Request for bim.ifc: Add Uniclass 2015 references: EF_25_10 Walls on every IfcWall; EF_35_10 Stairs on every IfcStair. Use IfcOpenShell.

First a look at what the model holds.

```python
import ifcopenshell

model = ifcopenshell.open("bim.ifc")
print(model.schema)
print("classifications:", [c.Name for c in model.by_type("IfcClassification")])
for ifc_class in ("IfcDoor", "IfcRoof", "IfcStair", "IfcWall", "IfcWindow"):
    print(ifc_class, len(model.by_type(ifc_class)))
```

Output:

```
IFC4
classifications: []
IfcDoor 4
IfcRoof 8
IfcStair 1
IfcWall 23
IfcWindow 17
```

```python
import ifcopenshell
import ifcopenshell.api.classification

model = ifcopenshell.open("bim.ifc")

system = ifcopenshell.api.classification.add_classification(model, classification="Uniclass 2015")

codes = {
    "IfcWall": ("EF_25_10", "Walls"),
    "IfcStair": ("EF_35_10", "Stairs"),
}
for ifc_class, (code, name) in codes.items():
    products = model.by_type(ifc_class)
    ifcopenshell.api.classification.add_reference(
        model, products=products, classification=system, identification=code, name=name
    )
    print(code, len(products))

model.write("bim_v2.ifc")
```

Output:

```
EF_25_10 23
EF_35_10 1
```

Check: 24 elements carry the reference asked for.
